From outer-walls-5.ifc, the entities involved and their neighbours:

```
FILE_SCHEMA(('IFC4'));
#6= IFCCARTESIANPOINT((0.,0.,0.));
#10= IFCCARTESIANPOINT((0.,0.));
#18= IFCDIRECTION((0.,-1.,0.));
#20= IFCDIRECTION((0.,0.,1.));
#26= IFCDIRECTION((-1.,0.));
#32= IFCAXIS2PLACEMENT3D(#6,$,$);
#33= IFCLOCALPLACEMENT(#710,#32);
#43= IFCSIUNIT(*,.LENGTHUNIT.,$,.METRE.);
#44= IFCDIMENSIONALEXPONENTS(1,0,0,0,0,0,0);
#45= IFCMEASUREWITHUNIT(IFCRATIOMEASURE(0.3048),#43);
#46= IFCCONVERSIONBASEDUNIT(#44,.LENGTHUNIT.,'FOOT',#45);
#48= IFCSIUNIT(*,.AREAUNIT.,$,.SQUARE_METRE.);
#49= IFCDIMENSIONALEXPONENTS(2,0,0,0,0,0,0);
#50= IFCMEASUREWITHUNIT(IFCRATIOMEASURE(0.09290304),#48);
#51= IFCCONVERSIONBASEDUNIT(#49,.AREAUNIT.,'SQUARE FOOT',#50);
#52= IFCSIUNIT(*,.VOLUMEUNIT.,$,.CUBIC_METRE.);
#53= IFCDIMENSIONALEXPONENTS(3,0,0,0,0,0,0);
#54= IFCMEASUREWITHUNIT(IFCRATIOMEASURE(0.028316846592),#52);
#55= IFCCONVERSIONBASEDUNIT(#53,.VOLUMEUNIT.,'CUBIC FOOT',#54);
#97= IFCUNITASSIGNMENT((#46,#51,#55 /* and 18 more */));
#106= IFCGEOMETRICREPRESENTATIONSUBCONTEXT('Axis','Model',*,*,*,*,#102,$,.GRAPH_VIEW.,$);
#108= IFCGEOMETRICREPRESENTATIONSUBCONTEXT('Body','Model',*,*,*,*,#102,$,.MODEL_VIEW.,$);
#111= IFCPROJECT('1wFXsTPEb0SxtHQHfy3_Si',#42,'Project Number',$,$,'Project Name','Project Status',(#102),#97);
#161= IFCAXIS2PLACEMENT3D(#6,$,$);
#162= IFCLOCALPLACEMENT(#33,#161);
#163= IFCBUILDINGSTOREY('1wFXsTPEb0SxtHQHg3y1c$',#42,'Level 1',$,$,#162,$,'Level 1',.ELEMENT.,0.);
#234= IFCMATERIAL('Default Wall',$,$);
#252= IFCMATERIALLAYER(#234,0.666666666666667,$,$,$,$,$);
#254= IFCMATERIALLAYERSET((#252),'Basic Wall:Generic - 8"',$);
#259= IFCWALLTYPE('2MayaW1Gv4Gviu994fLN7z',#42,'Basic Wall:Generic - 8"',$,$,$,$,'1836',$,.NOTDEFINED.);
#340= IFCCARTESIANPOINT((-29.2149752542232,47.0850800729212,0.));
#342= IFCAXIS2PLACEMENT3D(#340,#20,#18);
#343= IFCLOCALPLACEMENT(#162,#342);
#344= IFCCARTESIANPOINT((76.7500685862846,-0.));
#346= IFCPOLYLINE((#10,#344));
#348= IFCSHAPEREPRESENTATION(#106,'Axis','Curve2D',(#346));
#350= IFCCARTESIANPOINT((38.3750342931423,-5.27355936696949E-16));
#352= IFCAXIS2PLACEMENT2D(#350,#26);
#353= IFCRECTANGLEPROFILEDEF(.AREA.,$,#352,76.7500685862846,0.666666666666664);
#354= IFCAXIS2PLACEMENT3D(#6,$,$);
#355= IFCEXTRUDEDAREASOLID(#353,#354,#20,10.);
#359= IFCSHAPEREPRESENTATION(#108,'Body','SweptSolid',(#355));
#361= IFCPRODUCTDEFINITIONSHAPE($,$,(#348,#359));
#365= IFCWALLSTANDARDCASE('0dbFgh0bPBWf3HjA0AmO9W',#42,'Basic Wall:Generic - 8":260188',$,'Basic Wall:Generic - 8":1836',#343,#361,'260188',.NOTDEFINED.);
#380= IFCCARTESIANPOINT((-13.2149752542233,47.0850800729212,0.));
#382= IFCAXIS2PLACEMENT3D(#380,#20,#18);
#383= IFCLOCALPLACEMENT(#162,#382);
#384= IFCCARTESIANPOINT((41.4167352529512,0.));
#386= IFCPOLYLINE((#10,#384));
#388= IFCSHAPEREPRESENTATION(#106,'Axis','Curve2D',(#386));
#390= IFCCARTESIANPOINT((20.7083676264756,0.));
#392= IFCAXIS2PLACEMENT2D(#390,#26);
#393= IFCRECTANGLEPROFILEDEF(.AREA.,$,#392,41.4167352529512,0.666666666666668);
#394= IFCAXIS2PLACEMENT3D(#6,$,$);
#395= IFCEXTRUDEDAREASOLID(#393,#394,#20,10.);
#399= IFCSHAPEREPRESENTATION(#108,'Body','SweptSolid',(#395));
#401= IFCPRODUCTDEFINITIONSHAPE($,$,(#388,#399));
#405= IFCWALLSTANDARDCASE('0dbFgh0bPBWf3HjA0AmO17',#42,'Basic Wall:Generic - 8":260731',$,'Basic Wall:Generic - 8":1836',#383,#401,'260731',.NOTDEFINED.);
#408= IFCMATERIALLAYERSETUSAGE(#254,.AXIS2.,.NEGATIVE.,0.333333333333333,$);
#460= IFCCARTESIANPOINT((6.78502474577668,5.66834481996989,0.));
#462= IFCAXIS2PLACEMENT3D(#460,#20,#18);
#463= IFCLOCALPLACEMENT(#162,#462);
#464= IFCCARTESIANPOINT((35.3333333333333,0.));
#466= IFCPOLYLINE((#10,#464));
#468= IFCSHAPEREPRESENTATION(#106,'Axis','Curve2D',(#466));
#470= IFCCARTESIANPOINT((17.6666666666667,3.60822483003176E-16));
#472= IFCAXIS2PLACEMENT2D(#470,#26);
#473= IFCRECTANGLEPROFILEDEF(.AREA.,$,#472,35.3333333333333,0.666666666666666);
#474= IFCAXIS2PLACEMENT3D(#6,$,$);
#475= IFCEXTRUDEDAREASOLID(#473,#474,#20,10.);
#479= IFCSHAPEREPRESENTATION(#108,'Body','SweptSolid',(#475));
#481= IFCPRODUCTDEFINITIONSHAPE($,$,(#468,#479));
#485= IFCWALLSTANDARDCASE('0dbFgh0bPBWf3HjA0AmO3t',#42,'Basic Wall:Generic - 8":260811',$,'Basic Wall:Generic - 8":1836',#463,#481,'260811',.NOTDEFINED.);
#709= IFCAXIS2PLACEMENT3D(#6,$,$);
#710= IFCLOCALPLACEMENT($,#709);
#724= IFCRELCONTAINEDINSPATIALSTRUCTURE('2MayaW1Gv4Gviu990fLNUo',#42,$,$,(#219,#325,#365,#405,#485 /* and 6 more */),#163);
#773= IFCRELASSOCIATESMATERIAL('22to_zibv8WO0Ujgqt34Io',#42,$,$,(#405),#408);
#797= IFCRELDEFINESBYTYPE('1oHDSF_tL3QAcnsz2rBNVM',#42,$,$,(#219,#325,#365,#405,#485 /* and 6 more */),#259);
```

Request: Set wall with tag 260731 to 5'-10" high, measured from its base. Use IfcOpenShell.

```python
import ifcopenshell
import ifcopenshell.geom
import ifcopenshell.util.representation
import ifcopenshell.util.shape
import ifcopenshell.util.unit

model = ifcopenshell.open("outer-walls-5.ifc")
unit_scale = ifcopenshell.util.unit.calculate_unit_scale(model)
settings = ifcopenshell.geom.settings()


def volume(element):
    """Net volume in cubic metres, openings subtracted."""
    shape = ifcopenshell.geom.create_shape(settings, element)
    return ifcopenshell.util.shape.get_volume(shape.geometry)


wall = model.by_id(405)
before = volume(wall)

body = ifcopenshell.util.representation.get_representation(wall, "Model", "Body")
solid = body.Items[0]
old_height = solid.Depth
solid.Depth = 70 * 0.0254 / unit_scale
after = volume(wall)

print(f"height {old_height:g} -> {solid.Depth:g}, volume {before:.3f} -> {after:.3f} m3")

model.write("outer-walls-5_v2.ifc")
```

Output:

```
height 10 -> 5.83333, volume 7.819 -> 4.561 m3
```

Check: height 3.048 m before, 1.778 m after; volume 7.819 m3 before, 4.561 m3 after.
